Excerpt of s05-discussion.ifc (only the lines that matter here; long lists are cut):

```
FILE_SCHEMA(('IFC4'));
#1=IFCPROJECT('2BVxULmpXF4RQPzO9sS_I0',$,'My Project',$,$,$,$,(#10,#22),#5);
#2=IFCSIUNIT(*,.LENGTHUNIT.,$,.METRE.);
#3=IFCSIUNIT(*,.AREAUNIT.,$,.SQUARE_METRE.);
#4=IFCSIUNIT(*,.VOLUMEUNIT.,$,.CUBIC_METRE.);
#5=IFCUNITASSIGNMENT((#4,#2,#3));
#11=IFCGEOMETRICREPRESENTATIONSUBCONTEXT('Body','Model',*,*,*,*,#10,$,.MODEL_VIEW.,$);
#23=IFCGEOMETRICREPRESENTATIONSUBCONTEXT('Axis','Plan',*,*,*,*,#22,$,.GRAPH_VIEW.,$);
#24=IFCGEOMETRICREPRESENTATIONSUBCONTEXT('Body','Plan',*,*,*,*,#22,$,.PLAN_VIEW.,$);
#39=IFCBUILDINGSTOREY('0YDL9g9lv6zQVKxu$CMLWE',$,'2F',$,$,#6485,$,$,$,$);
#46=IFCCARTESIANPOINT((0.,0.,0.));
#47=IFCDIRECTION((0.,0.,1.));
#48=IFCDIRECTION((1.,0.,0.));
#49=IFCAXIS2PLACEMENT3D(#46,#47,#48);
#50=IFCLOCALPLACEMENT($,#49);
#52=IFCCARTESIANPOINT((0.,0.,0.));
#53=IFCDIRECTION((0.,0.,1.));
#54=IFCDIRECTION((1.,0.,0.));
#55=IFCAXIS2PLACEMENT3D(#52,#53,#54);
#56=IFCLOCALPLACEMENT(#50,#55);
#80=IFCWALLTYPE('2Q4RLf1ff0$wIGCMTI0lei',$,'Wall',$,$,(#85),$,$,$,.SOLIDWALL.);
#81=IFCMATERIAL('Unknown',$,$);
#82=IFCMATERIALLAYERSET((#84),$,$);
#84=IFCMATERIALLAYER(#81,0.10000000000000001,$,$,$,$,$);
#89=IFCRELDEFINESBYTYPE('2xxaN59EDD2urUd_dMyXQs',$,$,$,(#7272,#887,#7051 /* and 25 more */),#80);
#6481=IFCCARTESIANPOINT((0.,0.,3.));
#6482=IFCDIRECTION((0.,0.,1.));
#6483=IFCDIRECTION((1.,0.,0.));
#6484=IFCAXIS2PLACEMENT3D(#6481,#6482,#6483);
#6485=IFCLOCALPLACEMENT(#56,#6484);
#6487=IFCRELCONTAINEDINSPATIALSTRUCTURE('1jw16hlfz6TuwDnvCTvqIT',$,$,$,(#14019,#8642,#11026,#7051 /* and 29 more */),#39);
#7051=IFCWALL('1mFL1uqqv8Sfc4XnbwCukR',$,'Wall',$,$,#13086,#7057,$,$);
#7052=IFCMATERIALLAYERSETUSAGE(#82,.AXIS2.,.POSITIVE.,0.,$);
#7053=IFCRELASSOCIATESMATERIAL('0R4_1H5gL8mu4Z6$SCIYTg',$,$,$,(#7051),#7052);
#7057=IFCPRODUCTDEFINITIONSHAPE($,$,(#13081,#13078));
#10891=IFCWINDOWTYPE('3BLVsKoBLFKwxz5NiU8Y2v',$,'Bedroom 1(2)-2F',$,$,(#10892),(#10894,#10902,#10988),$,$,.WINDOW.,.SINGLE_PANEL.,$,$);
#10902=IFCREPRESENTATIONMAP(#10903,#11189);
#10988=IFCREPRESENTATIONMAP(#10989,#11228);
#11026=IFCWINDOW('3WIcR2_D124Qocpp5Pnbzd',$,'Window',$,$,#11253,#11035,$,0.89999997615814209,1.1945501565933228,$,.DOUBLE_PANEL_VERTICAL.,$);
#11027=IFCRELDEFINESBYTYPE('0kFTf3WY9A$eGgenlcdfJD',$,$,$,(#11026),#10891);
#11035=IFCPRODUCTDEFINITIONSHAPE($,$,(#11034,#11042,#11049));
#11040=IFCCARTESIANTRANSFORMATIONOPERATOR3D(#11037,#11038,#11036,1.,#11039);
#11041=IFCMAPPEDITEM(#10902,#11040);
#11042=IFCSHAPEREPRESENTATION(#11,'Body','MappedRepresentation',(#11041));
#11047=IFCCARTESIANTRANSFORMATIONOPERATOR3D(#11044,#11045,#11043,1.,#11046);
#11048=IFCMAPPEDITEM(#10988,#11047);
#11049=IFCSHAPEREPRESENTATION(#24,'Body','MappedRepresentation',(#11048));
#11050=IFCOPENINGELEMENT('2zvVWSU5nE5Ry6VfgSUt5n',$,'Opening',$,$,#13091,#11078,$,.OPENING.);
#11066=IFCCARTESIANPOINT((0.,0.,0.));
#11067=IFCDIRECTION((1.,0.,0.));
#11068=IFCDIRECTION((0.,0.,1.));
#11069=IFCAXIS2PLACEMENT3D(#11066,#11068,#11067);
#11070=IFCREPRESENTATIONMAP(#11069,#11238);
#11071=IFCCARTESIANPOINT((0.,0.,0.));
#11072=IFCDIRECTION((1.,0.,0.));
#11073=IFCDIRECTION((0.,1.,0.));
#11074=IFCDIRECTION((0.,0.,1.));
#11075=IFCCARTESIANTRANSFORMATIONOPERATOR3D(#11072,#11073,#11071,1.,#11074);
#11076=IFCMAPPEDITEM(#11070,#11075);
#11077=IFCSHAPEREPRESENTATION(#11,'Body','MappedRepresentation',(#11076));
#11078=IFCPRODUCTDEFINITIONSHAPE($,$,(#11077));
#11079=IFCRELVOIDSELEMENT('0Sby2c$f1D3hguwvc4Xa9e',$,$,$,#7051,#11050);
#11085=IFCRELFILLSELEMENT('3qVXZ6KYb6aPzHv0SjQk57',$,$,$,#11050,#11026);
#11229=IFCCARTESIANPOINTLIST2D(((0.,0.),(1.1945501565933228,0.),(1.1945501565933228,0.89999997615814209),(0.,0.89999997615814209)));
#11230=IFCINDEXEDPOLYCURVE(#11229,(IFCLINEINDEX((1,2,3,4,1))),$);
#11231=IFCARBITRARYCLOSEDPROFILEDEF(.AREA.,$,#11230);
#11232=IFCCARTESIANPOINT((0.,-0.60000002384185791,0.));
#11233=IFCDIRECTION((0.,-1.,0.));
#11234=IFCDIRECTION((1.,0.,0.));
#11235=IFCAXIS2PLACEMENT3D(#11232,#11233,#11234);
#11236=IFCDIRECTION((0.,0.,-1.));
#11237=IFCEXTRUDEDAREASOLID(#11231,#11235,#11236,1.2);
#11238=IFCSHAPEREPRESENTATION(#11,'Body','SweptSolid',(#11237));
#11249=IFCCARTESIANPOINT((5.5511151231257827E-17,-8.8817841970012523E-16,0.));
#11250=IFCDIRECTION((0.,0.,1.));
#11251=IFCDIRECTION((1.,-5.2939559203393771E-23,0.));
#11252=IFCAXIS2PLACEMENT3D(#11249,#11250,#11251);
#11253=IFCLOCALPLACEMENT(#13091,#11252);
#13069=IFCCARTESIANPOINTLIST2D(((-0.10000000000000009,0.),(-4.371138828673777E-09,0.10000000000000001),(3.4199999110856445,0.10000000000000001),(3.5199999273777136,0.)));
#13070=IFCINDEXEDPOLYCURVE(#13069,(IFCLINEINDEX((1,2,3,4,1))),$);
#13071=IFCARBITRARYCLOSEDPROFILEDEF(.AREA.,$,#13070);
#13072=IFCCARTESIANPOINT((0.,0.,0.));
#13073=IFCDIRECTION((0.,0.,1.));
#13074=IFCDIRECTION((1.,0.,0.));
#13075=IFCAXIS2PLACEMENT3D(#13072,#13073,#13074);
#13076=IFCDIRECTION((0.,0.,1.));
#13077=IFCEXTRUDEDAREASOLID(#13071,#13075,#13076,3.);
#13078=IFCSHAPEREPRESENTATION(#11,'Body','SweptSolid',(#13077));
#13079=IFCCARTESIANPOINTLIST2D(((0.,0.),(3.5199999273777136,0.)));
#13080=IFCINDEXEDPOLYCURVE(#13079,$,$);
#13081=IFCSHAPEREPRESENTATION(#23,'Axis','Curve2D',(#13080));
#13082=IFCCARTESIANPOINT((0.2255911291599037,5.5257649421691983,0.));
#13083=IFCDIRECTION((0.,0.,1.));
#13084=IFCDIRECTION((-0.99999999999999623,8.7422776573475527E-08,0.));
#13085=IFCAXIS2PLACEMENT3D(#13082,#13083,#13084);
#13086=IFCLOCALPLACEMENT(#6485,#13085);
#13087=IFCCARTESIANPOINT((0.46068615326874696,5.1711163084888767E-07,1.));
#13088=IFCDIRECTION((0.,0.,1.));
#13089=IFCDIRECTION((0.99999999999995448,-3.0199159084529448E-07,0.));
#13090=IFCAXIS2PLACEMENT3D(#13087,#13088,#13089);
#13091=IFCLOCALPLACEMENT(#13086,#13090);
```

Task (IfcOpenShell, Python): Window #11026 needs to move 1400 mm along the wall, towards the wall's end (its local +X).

```python
import ifcopenshell
import ifcopenshell.api.geometry
import ifcopenshell.util.placement
import ifcopenshell.util.unit

model = ifcopenshell.open("s05-discussion.ifc")
unit_scale = ifcopenshell.util.unit.calculate_unit_scale(model)

window = model.by_guid("3WIcR2_D124Qocpp5Pnbzd")
opening = window.FillsVoids[0].RelatingOpeningElement
wall = opening.VoidsElements[0].RelatingBuildingElement

wall_matrix = ifcopenshell.util.placement.get_local_placement(wall.ObjectPlacement)
shift = wall_matrix[:3, 0] * 1.4 / unit_scale
before = ifcopenshell.util.placement.get_local_placement(window.ObjectPlacement)[:3, 3].copy()

# The window is placed relative to its opening, so it follows when the opening moves.
matrix = ifcopenshell.util.placement.get_local_placement(opening.ObjectPlacement)
matrix[:3, 3] += shift
ifcopenshell.api.geometry.edit_object_placement(
    model, product=opening, matrix=matrix, is_si=False, should_transform_children=True
)

after = ifcopenshell.util.placement.get_local_placement(window.ObjectPlacement)[:3, 3]
print("window moved by", (after - before).round(3) + 0.0)

model.write("s05-discussion_edited.ifc")
```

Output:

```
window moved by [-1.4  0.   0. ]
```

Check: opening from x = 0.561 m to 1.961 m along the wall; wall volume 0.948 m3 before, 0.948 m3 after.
